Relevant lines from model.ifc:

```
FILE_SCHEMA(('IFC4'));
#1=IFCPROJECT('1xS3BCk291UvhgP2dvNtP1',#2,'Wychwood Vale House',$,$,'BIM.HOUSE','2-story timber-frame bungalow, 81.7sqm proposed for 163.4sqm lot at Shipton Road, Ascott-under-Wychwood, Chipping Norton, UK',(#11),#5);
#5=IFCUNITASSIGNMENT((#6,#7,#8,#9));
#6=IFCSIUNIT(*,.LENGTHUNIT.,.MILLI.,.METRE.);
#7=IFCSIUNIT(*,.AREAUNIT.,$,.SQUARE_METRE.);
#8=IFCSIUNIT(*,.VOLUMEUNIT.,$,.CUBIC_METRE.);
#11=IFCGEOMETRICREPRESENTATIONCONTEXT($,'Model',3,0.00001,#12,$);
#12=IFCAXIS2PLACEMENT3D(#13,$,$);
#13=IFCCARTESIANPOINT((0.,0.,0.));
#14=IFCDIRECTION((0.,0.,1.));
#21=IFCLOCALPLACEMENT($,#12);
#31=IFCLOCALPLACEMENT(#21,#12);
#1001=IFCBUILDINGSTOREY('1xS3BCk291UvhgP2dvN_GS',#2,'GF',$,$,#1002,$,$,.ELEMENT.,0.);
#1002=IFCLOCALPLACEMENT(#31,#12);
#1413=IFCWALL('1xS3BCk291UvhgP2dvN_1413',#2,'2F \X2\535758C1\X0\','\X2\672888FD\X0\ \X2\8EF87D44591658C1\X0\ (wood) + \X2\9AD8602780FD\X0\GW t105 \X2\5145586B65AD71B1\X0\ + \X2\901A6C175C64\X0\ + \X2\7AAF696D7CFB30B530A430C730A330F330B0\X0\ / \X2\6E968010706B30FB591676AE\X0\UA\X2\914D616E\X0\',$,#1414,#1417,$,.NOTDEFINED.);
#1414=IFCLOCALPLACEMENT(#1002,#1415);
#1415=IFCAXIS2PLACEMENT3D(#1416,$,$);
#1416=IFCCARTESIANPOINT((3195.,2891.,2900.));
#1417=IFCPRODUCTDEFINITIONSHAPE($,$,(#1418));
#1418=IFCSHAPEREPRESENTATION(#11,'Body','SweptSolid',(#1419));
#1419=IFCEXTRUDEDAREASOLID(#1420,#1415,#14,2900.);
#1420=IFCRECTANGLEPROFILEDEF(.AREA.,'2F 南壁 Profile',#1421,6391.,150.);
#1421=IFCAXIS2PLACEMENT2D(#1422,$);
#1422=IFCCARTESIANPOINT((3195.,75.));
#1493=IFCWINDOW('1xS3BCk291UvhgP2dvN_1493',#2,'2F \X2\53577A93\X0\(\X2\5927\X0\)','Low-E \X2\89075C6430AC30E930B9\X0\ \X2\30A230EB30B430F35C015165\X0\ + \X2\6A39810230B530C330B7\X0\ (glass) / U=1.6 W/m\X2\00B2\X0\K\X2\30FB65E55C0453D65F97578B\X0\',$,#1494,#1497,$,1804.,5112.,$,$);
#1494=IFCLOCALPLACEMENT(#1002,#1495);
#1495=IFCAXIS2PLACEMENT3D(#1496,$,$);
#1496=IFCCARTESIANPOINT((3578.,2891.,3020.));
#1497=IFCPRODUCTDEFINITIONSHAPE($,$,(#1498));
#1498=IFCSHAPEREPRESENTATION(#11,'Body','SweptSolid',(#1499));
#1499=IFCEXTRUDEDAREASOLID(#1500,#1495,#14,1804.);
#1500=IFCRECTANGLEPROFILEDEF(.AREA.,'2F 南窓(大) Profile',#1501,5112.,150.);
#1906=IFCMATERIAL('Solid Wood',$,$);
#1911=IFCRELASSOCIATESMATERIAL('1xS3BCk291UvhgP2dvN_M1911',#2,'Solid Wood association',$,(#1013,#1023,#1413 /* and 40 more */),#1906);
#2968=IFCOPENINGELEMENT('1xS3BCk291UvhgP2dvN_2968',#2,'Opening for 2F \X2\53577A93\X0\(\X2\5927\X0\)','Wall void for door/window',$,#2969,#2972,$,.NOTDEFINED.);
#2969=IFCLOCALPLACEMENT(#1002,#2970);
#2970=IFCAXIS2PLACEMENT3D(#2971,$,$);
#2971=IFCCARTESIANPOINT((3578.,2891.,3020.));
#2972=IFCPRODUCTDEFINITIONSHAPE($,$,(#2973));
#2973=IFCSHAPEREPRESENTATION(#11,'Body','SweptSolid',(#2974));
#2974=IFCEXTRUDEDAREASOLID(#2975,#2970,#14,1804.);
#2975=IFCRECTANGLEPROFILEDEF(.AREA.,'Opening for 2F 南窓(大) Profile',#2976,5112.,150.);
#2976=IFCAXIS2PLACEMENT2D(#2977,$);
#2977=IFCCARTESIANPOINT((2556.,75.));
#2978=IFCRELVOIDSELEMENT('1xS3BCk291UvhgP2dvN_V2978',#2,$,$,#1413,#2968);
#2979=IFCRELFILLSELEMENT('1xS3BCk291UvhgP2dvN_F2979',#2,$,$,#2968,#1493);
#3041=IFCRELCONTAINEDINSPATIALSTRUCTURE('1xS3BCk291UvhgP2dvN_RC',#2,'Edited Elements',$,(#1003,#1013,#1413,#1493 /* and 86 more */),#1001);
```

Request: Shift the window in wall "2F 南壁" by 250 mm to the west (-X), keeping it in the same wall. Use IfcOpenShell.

```python
import ifcopenshell
import ifcopenshell.api.geometry
import ifcopenshell.util.placement
import ifcopenshell.util.unit

model = ifcopenshell.open("model.ifc")
unit_scale = ifcopenshell.util.unit.calculate_unit_scale(model)

window = model.by_id(1493)
opening = window.FillsVoids[0].RelatingOpeningElement
wall = opening.VoidsElements[0].RelatingBuildingElement

wall_matrix = ifcopenshell.util.placement.get_local_placement(wall.ObjectPlacement)
shift = wall_matrix[:3, 0] * -0.25 / unit_scale
before = ifcopenshell.util.placement.get_local_placement(window.ObjectPlacement)[:3, 3].copy()

# The window is not placed relative to its opening, so move both.
for product in (opening, window):
    matrix = ifcopenshell.util.placement.get_local_placement(product.ObjectPlacement)
    matrix[:3, 3] += shift
    ifcopenshell.api.geometry.edit_object_placement(model, product=product, matrix=matrix, is_si=False)

after = ifcopenshell.util.placement.get_local_placement(window.ObjectPlacement)[:3, 3]
print("window moved by", (after - before).round(3) + 0.0)

model.write("model-out.ifc")
```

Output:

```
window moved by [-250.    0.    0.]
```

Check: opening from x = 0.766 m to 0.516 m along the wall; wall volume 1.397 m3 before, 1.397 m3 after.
